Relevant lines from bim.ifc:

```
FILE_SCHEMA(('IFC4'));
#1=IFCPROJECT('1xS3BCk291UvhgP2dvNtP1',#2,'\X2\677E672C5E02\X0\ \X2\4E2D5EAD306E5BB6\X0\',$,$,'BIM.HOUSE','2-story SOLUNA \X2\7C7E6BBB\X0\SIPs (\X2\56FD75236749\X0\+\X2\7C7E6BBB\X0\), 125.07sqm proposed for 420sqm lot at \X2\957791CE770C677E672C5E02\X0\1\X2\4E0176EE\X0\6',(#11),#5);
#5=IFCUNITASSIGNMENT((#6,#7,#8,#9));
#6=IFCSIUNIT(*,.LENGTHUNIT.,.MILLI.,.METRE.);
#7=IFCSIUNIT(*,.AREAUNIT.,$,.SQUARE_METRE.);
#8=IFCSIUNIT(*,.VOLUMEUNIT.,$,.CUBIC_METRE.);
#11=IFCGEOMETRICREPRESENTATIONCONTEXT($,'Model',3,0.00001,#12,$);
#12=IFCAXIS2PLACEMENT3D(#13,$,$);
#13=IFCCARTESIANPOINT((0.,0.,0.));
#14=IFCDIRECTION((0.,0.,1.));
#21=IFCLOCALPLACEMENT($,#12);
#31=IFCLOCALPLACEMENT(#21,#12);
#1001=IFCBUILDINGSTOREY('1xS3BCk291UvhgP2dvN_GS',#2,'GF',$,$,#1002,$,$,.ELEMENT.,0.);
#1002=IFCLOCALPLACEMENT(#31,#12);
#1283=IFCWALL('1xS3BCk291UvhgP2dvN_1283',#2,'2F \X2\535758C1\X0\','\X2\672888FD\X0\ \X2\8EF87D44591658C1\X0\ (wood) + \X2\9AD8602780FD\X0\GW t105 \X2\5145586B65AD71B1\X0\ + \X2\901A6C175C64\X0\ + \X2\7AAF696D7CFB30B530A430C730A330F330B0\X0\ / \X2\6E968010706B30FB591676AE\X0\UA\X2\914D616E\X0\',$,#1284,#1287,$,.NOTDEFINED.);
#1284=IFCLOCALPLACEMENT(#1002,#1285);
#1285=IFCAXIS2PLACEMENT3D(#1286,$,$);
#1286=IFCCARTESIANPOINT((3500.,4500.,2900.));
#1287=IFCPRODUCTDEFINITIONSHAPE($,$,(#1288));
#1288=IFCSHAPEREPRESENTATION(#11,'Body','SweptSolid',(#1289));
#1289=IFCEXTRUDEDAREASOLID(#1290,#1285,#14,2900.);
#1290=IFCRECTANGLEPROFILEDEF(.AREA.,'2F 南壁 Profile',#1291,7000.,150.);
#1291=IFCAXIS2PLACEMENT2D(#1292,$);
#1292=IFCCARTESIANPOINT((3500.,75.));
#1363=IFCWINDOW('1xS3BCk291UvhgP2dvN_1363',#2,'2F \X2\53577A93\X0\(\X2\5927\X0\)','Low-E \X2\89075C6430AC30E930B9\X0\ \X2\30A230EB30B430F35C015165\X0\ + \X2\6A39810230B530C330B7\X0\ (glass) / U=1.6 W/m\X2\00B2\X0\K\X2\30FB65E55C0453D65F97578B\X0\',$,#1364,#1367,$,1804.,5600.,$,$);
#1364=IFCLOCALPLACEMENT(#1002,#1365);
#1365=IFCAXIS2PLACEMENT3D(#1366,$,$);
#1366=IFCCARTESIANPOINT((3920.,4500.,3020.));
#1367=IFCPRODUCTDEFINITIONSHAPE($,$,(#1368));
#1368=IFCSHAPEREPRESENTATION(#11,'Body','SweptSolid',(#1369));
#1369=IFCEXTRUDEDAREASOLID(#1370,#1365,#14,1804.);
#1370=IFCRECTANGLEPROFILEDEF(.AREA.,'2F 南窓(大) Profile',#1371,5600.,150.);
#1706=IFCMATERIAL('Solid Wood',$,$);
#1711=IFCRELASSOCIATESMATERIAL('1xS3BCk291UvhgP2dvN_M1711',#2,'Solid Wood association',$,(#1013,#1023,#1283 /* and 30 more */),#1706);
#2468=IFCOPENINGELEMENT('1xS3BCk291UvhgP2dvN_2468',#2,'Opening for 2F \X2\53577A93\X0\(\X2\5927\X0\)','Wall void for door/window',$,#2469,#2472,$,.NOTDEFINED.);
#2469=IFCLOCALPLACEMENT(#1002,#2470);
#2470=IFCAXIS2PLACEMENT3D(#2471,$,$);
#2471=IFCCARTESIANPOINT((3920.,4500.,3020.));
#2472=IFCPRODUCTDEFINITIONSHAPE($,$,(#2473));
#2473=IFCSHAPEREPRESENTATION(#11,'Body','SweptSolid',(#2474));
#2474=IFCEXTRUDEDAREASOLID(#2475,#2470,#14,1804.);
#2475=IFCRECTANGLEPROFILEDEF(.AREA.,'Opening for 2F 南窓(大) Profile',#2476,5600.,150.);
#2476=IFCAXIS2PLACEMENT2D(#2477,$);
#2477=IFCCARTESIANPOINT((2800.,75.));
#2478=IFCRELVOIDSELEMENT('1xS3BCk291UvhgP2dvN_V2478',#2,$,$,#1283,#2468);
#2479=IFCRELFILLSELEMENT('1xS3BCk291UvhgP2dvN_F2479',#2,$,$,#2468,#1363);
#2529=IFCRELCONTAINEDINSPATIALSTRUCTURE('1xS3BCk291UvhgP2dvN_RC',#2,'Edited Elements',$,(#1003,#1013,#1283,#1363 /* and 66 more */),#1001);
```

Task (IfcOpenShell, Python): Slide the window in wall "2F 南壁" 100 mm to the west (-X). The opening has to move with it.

```python
import ifcopenshell
import ifcopenshell.api.geometry
import ifcopenshell.util.placement
import ifcopenshell.util.unit

model = ifcopenshell.open("bim.ifc")
unit_scale = ifcopenshell.util.unit.calculate_unit_scale(model)

window = model.by_guid("1xS3BCk291UvhgP2dvN_1363")
opening = window.FillsVoids[0].RelatingOpeningElement
wall = opening.VoidsElements[0].RelatingBuildingElement

wall_matrix = ifcopenshell.util.placement.get_local_placement(wall.ObjectPlacement)
shift = wall_matrix[:3, 0] * -0.1 / unit_scale
before = ifcopenshell.util.placement.get_local_placement(window.ObjectPlacement)[:3, 3].copy()

# The window is not placed relative to its opening, so move both.
for product in (opening, window):
    matrix = ifcopenshell.util.placement.get_local_placement(product.ObjectPlacement)
    matrix[:3, 3] += shift
    ifcopenshell.api.geometry.edit_object_placement(model, product=product, matrix=matrix, is_si=False)

after = ifcopenshell.util.placement.get_local_placement(window.ObjectPlacement)[:3, 3]
print("window moved by", (after - before).round(3) + 0.0)

model.write("bim_v2.ifc")
```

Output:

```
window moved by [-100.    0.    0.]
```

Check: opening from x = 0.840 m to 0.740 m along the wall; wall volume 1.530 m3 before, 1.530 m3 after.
